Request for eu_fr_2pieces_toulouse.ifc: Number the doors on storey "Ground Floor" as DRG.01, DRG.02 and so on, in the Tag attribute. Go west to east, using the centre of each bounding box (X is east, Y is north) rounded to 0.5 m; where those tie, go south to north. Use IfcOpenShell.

First a look at what the model holds.

```python
import ifcopenshell
import ifcopenshell.util.element
import ifcopenshell.util.placement

model = ifcopenshell.open("eu_fr_2pieces_toulouse.ifc")
print(model.schema)
storey = next(s for s in model.by_type("IfcBuildingStorey") if s.Name == "Ground Floor")
doors = [e for e in ifcopenshell.util.element.get_decomposition(storey) if e.is_a("IfcDoor")]
for e in sorted(doors, key=lambda e: e.id()):
    origin = ifcopenshell.util.placement.get_local_placement(e.ObjectPlacement)[:3, 3]
    print(e.id(), e.Tag, e.Name, origin.round(2) + 0.0, sep=" | ")
```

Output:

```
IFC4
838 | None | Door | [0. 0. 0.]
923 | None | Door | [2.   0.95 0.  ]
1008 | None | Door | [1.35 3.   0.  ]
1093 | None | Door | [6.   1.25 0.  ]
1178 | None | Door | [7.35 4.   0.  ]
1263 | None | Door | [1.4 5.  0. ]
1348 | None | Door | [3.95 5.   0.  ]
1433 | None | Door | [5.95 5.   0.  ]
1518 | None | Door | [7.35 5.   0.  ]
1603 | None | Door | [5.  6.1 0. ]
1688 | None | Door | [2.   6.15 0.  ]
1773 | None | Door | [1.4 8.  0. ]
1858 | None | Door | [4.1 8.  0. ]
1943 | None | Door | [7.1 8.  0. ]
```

```python
import ifcopenshell
import ifcopenshell.geom
import ifcopenshell.util.element
import ifcopenshell.util.shape

model = ifcopenshell.open("eu_fr_2pieces_toulouse.ifc")
settings = ifcopenshell.geom.settings()
settings.set("use-world-coords", True)


def centre(element):
    shape = ifcopenshell.geom.create_shape(settings, element)
    return ifcopenshell.util.shape.get_bbox_centroid(shape.geometry)


storey = next(s for s in model.by_type("IfcBuildingStorey") if s.Name == "Ground Floor")
doors = [e for e in ifcopenshell.util.element.get_decomposition(storey) if e.is_a("IfcDoor")]

# Insertion points can sit at a corner or the storey origin, so sort by the geometry (in metres).
centres = {e: centre(e) for e in doors}
doors.sort(key=lambda e: (round(centres[e][0] / 0.5), centres[e][1]))

for i, e in enumerate(doors, start=1):
    number = f"DRG.{i:02d}"
    e.Tag = number
    print(e.id(), number)

model.write("eu_fr_2pieces_toulouse_v2.ifc")
```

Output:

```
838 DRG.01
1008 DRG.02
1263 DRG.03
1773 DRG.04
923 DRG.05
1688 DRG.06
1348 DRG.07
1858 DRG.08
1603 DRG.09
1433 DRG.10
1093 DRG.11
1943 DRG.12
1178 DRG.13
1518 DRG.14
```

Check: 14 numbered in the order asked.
